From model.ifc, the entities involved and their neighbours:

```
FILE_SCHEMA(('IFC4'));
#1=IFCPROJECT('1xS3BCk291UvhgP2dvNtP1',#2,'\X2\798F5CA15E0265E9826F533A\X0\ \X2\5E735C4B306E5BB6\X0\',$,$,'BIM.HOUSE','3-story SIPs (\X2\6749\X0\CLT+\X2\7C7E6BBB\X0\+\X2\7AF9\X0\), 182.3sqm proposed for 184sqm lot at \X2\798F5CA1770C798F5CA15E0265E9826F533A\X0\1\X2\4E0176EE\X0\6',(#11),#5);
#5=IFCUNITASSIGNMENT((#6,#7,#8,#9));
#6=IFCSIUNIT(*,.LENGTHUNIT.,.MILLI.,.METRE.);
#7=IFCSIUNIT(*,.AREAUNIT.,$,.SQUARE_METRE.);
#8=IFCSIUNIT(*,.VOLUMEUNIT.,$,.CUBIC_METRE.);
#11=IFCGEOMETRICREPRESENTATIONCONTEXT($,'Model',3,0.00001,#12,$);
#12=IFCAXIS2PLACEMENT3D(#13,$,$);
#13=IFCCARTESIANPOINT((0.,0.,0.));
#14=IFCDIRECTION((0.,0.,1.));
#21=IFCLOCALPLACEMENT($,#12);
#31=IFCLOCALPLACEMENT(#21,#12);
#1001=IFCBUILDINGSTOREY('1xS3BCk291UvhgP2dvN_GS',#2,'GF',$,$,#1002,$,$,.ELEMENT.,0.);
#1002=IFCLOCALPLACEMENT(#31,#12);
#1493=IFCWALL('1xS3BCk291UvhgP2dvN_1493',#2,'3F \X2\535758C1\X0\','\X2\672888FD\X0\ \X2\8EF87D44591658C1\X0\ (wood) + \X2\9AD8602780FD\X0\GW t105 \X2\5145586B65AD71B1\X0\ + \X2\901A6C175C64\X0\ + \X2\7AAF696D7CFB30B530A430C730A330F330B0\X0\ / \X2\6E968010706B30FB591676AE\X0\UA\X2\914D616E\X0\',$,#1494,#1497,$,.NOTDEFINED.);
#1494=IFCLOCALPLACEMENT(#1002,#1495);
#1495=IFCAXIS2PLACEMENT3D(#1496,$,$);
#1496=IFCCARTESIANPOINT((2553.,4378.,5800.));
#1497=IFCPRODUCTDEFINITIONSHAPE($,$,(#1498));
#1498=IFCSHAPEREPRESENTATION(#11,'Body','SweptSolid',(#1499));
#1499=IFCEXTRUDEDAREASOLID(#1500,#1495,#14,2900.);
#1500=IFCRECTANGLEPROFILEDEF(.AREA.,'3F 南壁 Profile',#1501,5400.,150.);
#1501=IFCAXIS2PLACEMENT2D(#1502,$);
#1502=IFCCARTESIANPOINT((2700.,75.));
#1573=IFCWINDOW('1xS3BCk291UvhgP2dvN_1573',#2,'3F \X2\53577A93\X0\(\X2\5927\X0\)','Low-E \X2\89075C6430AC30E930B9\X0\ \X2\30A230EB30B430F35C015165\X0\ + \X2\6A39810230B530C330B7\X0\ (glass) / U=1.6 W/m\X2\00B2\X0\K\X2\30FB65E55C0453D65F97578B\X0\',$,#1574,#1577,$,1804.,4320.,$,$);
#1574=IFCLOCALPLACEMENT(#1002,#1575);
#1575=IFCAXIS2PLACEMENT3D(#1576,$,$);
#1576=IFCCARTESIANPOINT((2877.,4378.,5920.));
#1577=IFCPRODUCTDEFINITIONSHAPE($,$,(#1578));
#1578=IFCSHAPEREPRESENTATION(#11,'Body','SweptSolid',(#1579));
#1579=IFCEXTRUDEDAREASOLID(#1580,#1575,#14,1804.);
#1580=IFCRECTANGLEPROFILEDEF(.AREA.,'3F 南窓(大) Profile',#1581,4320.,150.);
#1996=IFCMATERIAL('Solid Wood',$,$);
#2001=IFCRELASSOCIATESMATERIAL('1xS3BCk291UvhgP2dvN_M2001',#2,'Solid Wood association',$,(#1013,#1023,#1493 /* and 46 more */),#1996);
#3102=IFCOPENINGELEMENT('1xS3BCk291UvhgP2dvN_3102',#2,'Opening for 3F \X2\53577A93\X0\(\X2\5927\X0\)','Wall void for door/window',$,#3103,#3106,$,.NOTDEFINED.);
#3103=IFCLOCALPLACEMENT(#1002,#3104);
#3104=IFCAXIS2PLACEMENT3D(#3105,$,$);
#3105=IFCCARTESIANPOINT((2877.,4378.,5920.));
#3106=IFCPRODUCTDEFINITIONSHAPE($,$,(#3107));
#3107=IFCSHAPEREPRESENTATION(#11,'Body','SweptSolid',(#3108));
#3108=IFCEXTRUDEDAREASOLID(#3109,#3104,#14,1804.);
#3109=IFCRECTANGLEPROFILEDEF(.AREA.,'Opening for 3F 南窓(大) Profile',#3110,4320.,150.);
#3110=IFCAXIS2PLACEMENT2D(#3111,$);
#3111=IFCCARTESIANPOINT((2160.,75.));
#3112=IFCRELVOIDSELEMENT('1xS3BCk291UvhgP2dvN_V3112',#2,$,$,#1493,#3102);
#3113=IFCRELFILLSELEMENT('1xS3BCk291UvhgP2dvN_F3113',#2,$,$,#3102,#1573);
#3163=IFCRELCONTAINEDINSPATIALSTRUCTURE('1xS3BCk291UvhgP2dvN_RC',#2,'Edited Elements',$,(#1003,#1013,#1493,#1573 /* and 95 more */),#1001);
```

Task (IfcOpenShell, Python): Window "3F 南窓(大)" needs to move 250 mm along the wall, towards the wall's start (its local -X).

```python
import ifcopenshell
import ifcopenshell.api.geometry
import ifcopenshell.util.placement
import ifcopenshell.util.unit

model = ifcopenshell.open("model.ifc")
unit_scale = ifcopenshell.util.unit.calculate_unit_scale(model)

window = model.by_guid("1xS3BCk291UvhgP2dvN_1573")
opening = window.FillsVoids[0].RelatingOpeningElement
wall = opening.VoidsElements[0].RelatingBuildingElement

wall_matrix = ifcopenshell.util.placement.get_local_placement(wall.ObjectPlacement)
shift = wall_matrix[:3, 0] * -0.25 / unit_scale
before = ifcopenshell.util.placement.get_local_placement(window.ObjectPlacement)[:3, 3].copy()

# The window is not placed relative to its opening, so move both.
for product in (opening, window):
    matrix = ifcopenshell.util.placement.get_local_placement(product.ObjectPlacement)
    matrix[:3, 3] += shift
    ifcopenshell.api.geometry.edit_object_placement(model, product=product, matrix=matrix, is_si=False)

after = ifcopenshell.util.placement.get_local_placement(window.ObjectPlacement)[:3, 3]
print("window moved by", (after - before).round(3) + 0.0)

model.write("model_rev.ifc")
```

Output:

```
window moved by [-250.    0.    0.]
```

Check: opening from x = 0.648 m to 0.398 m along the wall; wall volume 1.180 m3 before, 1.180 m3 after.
